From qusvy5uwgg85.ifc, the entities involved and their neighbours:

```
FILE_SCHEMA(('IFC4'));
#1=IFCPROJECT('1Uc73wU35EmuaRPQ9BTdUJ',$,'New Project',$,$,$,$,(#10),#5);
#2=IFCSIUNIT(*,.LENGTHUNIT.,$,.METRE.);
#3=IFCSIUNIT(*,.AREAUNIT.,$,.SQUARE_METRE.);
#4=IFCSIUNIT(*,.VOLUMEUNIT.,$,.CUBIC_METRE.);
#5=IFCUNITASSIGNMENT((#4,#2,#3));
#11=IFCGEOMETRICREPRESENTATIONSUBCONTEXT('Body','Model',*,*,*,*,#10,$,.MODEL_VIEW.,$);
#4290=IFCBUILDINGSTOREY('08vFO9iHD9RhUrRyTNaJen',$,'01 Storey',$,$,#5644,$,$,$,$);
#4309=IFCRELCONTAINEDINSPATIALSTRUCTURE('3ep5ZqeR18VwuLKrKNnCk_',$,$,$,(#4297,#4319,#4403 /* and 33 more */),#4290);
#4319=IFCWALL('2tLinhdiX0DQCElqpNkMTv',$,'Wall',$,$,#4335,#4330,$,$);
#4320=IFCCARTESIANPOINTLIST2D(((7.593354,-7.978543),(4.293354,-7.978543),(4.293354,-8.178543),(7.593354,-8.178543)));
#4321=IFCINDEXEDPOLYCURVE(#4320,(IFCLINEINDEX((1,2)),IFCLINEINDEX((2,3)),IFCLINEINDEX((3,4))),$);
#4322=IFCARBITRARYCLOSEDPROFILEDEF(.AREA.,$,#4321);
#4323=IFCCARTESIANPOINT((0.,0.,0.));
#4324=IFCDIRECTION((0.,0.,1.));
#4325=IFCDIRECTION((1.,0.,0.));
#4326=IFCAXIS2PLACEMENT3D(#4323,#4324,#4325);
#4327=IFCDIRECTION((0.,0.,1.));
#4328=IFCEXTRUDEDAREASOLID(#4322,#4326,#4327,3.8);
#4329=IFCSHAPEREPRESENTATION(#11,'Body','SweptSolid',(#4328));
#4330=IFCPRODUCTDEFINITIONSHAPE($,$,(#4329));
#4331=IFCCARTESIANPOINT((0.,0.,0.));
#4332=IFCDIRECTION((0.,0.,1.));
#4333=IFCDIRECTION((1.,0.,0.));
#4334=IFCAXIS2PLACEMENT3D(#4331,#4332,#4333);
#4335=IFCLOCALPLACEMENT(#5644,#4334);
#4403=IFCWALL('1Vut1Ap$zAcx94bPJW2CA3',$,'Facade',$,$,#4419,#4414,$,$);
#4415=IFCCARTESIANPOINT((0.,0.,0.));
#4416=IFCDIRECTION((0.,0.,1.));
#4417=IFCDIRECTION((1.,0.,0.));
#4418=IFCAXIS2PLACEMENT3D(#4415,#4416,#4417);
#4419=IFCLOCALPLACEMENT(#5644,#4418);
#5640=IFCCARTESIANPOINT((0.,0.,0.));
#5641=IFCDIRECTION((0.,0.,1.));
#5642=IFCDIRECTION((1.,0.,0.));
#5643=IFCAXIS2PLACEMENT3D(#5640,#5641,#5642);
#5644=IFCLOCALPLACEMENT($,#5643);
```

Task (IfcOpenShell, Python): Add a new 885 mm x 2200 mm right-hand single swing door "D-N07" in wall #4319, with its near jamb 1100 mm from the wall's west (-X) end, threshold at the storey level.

```python
import numpy as np
import ifcopenshell
import ifcopenshell.api.feature
import ifcopenshell.api.geometry
import ifcopenshell.api.root
import ifcopenshell.api.spatial
import ifcopenshell.geom
import ifcopenshell.util.element
import ifcopenshell.util.placement
import ifcopenshell.util.representation
import ifcopenshell.util.shape
import ifcopenshell.util.unit

model = ifcopenshell.open("qusvy5uwgg85.ifc")
unit_scale = ifcopenshell.util.unit.calculate_unit_scale(model)
settings = ifcopenshell.geom.settings()


def volume(element):
    """Net volume in cubic metres, openings subtracted."""
    shape = ifcopenshell.geom.create_shape(settings, element)
    return ifcopenshell.util.shape.get_volume(shape.geometry)


wall = model.by_guid("2tLinhdiX0DQCElqpNkMTv")
storey = ifcopenshell.util.element.get_container(wall, ifc_class="IfcBuildingStorey")
context = ifcopenshell.util.representation.get_context(model, "Model", "Body", "MODEL_VIEW")
before = volume(wall)

width, height, from_end, sill = 0.885, 2.2, 1.1, 0.0  # metres

# The wall runs along its own X axis, and the end named is its -X end.
wall_shape = ifcopenshell.geom.create_shape(settings, wall)
x, y, z = ifcopenshell.util.shape.get_vertices(wall_shape.geometry).T
start = x.min() + from_end
face, thickness = float(y.min()), float(y.max() - y.min())
wall_matrix = ifcopenshell.util.placement.get_local_placement(wall.ObjectPlacement)
level = ifcopenshell.util.placement.get_local_placement(storey.ObjectPlacement)[2, 3]


def in_wall(x, y):
    """Placement at x, y metres in the wall's axes, at sill height."""
    matrix = wall_matrix.copy()
    matrix[:, 3] = wall_matrix @ np.array([x / unit_scale, y / unit_scale, 0.0, 1.0])
    matrix[2, 3] = level + sill / unit_scale
    return matrix


# Opening: a box that overshoots both wall faces by 50 mm.
opening = ifcopenshell.api.root.create_entity(model, ifc_class="IfcOpeningElement", predefined_type="OPENING")
box = ifcopenshell.api.geometry.add_wall_representation(
    model, context=context, length=width, height=height, thickness=thickness + 0.1
)
ifcopenshell.api.geometry.assign_representation(model, product=opening, representation=box)
ifcopenshell.api.geometry.edit_object_placement(model, product=opening, matrix=in_wall(start, face - 0.05), is_si=False)
ifcopenshell.api.feature.add_feature(model, feature=opening, element=wall)

door = ifcopenshell.api.root.create_entity(model, ifc_class="IfcDoor", name="D-N07", predefined_type="DOOR")
door.OverallWidth, door.OverallHeight = width / unit_scale, height / unit_scale
door.OperationType = "SINGLE_SWING_RIGHT"
body = ifcopenshell.api.geometry.add_door_representation(
    model,
    context=context,
    overall_width=door.OverallWidth,
    overall_height=door.OverallHeight,
    operation_type="SINGLE_SWING_RIGHT",
    lining_properties={"LiningDepth": thickness / unit_scale, "ThresholdDepth": thickness / unit_scale},
)
ifcopenshell.api.geometry.assign_representation(model, product=door, representation=body)
ifcopenshell.api.spatial.assign_container(model, products=[door], relating_structure=storey)
ifcopenshell.api.feature.add_filling(model, opening=opening, element=door)

# The lining spans the wall, so the door starts at the wall face.
ifcopenshell.api.geometry.edit_object_placement(model, product=door, matrix=in_wall(start, face), is_si=False)

after = volume(wall)

print(f"wall volume {before:.3f} -> {after:.3f} m3")

model.write("qusvy5uwgg85_updated.ifc")
```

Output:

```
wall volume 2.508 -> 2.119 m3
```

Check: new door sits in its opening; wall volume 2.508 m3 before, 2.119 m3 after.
